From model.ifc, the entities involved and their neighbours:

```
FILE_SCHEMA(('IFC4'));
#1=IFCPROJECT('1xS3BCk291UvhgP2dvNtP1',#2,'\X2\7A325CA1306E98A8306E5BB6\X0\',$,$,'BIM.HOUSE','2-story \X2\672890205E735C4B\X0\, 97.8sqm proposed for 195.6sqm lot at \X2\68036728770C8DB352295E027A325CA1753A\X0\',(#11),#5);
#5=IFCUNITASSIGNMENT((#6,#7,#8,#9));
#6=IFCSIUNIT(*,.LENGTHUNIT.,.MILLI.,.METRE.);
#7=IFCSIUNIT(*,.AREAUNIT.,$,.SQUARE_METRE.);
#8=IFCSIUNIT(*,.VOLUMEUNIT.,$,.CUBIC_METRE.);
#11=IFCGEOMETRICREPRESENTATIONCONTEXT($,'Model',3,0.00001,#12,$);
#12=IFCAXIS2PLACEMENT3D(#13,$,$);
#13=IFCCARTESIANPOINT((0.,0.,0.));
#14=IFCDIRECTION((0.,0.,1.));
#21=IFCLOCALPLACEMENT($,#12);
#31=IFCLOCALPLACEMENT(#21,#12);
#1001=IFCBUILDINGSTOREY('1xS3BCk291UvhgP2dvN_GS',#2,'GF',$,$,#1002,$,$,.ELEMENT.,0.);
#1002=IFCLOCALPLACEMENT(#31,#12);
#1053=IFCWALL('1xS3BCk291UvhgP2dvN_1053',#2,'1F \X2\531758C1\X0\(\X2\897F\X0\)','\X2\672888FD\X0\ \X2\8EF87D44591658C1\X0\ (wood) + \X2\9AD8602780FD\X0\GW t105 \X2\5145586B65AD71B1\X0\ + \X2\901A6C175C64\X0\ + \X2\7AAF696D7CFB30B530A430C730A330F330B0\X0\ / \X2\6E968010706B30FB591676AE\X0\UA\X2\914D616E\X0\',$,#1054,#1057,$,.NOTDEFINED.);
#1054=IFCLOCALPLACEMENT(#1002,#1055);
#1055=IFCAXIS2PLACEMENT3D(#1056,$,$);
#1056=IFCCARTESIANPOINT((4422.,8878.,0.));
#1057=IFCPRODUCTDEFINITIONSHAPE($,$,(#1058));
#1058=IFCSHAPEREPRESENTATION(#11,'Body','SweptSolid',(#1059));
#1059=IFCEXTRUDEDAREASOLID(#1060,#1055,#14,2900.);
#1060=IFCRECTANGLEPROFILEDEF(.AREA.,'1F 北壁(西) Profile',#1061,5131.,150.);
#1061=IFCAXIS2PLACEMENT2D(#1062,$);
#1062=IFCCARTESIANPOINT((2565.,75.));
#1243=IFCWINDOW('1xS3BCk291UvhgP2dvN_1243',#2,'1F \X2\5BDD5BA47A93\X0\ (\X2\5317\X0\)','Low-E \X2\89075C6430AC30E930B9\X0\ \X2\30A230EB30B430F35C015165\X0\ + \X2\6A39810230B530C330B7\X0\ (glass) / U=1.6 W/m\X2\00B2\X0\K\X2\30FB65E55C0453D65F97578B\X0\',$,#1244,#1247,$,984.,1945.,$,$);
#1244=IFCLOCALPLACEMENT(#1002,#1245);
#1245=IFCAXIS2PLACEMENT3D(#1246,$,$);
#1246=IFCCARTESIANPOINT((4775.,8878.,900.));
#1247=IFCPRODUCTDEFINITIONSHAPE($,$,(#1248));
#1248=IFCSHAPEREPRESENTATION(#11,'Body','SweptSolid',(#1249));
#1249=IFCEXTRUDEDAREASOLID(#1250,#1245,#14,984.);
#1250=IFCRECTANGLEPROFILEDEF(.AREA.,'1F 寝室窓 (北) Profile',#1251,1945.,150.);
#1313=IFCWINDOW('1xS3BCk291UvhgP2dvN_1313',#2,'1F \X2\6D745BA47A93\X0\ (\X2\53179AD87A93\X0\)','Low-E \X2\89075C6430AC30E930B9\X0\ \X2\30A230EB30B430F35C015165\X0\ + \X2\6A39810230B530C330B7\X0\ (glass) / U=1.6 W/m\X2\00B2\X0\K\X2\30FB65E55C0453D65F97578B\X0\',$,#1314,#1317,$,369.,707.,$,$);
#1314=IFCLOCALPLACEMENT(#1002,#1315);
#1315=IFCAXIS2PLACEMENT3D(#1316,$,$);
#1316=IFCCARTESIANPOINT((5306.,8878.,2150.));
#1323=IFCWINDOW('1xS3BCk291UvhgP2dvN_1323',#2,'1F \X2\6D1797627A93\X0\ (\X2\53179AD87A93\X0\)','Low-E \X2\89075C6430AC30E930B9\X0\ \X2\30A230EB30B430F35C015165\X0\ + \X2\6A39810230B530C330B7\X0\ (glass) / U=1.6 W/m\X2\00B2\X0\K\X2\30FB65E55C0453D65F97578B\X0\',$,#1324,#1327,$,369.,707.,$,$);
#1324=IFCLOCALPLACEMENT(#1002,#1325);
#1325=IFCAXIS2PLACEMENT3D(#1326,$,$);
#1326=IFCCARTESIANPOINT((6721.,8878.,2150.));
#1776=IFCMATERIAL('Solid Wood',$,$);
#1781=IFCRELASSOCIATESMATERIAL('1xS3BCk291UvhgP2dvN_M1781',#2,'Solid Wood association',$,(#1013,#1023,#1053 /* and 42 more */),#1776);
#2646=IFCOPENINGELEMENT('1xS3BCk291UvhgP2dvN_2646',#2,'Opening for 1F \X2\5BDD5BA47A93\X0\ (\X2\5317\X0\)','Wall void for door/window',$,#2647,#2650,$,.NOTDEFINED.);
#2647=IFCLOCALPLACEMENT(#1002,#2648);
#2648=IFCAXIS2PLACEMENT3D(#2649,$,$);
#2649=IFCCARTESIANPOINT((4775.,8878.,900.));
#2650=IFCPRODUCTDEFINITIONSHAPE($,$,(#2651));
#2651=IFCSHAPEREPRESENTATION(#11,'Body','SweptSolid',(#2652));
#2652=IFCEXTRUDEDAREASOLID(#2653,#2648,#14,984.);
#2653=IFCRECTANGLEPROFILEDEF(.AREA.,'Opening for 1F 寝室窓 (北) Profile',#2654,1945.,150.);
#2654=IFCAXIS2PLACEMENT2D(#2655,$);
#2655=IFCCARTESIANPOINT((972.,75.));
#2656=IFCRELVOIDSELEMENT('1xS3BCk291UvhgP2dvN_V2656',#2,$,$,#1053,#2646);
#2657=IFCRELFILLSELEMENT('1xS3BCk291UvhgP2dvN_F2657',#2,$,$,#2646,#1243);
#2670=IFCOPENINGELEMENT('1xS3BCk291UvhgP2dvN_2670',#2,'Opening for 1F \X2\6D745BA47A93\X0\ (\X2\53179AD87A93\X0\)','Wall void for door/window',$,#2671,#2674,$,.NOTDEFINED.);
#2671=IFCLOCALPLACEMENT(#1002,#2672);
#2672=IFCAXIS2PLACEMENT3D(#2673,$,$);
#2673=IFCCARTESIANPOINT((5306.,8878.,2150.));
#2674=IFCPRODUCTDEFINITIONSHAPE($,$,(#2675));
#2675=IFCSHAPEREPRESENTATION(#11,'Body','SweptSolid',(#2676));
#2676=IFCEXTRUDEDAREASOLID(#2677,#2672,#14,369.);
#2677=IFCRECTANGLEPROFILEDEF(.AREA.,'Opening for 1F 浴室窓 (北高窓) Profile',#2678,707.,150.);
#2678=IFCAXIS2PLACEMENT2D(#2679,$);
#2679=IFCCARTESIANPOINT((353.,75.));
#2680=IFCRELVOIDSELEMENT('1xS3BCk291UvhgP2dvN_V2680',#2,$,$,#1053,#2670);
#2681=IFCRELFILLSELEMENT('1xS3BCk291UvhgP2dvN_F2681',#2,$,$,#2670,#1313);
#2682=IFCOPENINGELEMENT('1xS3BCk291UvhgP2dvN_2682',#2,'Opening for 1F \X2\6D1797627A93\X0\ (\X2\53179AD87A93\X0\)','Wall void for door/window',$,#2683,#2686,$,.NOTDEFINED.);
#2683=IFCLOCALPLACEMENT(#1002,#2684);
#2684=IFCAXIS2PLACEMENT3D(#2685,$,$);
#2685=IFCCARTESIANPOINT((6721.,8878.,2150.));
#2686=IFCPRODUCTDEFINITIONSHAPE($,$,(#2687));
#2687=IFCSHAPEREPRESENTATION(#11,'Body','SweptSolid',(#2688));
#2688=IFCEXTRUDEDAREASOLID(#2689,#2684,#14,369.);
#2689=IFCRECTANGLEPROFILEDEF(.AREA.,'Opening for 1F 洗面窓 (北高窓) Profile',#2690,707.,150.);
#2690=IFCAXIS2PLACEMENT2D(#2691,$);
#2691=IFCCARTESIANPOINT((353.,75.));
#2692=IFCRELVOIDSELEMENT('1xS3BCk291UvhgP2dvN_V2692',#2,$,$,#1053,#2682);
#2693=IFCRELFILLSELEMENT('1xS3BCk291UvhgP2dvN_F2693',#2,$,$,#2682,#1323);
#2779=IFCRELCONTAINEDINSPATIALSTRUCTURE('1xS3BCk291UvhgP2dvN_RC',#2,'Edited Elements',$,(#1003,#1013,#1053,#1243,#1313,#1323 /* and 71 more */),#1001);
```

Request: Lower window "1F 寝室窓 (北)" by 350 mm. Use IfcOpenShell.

```python
import numpy as np
import ifcopenshell
import ifcopenshell.api.geometry
import ifcopenshell.util.placement
import ifcopenshell.util.unit

model = ifcopenshell.open("model.ifc")
unit_scale = ifcopenshell.util.unit.calculate_unit_scale(model)

window = model.by_id(1243)
opening = window.FillsVoids[0].RelatingOpeningElement
dz = -350.0

shift = np.array([0.0, 0.0, dz])
# The window is not placed relative to its opening, so move both.
for product in (opening, window):
    matrix = ifcopenshell.util.placement.get_local_placement(product.ObjectPlacement)
    matrix[:3, 3] += shift
    ifcopenshell.api.geometry.edit_object_placement(model, product=product, matrix=matrix, is_si=False)

print(f"moved by {dz * unit_scale:+.3f} m")

model.write("model_rev.ifc")
```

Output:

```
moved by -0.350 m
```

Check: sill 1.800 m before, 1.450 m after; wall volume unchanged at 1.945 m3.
